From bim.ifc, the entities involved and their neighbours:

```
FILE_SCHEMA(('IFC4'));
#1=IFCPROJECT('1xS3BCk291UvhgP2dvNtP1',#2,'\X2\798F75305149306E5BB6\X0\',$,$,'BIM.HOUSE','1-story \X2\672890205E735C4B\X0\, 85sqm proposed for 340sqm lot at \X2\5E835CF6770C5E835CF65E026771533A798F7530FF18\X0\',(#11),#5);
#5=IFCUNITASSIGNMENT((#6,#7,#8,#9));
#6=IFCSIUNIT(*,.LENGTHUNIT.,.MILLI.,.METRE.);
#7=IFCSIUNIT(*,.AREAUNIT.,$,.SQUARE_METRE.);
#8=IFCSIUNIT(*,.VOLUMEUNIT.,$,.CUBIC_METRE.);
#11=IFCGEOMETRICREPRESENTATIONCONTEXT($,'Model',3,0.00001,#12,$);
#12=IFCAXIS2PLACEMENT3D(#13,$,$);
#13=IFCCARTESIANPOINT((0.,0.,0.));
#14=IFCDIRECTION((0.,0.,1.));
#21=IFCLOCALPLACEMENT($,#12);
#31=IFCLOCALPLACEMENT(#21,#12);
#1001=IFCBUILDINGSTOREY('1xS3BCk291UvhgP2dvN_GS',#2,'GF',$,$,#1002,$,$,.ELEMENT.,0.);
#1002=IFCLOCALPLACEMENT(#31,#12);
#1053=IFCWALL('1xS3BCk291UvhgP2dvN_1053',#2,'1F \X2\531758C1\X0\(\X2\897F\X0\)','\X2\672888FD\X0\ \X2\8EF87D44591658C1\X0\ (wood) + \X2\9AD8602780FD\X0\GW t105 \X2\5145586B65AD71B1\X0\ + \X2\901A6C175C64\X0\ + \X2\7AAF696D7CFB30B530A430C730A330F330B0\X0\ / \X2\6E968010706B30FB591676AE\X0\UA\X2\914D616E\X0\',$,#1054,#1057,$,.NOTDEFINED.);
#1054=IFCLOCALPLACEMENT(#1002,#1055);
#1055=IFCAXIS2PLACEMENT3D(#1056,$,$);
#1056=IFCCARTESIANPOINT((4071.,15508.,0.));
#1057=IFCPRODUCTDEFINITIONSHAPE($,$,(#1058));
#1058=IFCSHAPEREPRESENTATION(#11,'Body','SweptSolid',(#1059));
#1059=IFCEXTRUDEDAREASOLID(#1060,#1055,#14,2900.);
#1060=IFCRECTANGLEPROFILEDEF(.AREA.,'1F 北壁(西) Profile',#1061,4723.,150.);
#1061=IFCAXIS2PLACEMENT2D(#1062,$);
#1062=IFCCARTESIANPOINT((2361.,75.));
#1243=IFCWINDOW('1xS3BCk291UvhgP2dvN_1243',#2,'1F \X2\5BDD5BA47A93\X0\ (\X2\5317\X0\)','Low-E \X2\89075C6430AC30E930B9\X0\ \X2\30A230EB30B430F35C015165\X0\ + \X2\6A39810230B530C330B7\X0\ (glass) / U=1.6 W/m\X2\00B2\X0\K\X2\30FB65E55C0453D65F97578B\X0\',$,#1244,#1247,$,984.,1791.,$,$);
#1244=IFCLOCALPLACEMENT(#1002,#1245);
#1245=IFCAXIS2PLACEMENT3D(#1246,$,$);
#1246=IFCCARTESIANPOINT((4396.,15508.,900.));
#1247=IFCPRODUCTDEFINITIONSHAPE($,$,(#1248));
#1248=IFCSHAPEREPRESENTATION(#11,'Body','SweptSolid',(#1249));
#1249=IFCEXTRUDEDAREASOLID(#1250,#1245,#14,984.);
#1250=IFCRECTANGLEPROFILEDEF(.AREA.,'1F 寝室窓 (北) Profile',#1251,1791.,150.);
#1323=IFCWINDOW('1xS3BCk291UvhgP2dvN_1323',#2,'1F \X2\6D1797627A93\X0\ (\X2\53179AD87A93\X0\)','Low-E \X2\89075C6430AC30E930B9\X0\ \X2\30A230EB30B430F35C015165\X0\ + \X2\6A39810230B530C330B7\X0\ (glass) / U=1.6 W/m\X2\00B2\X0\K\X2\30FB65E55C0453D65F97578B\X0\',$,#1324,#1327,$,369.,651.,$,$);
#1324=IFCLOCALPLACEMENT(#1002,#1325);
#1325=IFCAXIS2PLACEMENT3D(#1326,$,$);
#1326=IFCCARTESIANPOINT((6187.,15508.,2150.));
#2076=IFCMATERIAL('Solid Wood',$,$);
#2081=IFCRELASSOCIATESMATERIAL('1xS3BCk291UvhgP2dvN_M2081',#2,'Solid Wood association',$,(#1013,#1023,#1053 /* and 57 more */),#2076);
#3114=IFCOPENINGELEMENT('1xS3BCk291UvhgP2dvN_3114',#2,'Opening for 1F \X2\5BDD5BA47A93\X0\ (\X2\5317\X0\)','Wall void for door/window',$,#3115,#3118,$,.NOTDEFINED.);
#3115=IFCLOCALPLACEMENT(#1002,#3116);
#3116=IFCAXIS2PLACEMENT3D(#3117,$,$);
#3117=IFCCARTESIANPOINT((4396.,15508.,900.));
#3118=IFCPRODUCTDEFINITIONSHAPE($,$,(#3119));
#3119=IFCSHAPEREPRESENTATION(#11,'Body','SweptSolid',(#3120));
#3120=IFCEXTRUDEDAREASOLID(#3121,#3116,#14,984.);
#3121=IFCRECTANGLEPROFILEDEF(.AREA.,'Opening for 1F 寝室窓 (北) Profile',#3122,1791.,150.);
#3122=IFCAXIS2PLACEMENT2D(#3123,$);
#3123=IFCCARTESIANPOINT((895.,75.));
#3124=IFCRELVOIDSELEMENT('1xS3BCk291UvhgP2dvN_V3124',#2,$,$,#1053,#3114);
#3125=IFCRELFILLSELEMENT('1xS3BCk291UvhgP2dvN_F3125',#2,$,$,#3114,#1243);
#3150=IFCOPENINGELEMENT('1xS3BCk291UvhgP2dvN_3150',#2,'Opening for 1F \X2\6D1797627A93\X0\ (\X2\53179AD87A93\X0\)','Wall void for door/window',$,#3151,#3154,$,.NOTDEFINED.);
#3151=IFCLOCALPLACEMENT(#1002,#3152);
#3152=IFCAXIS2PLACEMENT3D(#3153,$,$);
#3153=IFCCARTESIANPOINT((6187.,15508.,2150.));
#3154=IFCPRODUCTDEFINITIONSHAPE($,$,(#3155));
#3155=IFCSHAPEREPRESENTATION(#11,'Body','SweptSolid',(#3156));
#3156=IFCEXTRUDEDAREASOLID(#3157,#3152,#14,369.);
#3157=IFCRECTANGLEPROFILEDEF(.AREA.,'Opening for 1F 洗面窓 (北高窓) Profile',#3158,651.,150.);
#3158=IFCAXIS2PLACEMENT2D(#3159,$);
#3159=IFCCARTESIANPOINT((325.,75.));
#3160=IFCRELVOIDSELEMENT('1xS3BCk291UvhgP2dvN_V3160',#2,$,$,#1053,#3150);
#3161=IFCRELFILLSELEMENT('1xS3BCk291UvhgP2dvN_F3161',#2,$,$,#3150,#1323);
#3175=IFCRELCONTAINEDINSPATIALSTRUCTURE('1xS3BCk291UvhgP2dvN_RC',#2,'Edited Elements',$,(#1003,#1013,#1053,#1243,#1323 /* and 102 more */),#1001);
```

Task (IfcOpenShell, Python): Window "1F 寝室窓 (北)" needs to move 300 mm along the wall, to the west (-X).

```python
import ifcopenshell
import ifcopenshell.api.geometry
import ifcopenshell.util.placement

model = ifcopenshell.open("bim.ifc")

window = model.by_guid("1xS3BCk291UvhgP2dvN_1243")
opening = window.FillsVoids[0].RelatingOpeningElement
wall = opening.VoidsElements[0].RelatingBuildingElement

wall_matrix = ifcopenshell.util.placement.get_local_placement(wall.ObjectPlacement)
shift = wall_matrix[:3, 0] * -300.0
before = ifcopenshell.util.placement.get_local_placement(window.ObjectPlacement)[:3, 3].copy()

# The window is not placed relative to its opening, so move both.
for product in (opening, window):
    matrix = ifcopenshell.util.placement.get_local_placement(product.ObjectPlacement)
    matrix[:3, 3] += shift
    ifcopenshell.api.geometry.edit_object_placement(model, product=product, matrix=matrix, is_si=False)

after = ifcopenshell.util.placement.get_local_placement(window.ObjectPlacement)[:3, 3]
print("window moved by", (after - before).round(3) + 0.0)

model.write("bim_v2.ifc")
```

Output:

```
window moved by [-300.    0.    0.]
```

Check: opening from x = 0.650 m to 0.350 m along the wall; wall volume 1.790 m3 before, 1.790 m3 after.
